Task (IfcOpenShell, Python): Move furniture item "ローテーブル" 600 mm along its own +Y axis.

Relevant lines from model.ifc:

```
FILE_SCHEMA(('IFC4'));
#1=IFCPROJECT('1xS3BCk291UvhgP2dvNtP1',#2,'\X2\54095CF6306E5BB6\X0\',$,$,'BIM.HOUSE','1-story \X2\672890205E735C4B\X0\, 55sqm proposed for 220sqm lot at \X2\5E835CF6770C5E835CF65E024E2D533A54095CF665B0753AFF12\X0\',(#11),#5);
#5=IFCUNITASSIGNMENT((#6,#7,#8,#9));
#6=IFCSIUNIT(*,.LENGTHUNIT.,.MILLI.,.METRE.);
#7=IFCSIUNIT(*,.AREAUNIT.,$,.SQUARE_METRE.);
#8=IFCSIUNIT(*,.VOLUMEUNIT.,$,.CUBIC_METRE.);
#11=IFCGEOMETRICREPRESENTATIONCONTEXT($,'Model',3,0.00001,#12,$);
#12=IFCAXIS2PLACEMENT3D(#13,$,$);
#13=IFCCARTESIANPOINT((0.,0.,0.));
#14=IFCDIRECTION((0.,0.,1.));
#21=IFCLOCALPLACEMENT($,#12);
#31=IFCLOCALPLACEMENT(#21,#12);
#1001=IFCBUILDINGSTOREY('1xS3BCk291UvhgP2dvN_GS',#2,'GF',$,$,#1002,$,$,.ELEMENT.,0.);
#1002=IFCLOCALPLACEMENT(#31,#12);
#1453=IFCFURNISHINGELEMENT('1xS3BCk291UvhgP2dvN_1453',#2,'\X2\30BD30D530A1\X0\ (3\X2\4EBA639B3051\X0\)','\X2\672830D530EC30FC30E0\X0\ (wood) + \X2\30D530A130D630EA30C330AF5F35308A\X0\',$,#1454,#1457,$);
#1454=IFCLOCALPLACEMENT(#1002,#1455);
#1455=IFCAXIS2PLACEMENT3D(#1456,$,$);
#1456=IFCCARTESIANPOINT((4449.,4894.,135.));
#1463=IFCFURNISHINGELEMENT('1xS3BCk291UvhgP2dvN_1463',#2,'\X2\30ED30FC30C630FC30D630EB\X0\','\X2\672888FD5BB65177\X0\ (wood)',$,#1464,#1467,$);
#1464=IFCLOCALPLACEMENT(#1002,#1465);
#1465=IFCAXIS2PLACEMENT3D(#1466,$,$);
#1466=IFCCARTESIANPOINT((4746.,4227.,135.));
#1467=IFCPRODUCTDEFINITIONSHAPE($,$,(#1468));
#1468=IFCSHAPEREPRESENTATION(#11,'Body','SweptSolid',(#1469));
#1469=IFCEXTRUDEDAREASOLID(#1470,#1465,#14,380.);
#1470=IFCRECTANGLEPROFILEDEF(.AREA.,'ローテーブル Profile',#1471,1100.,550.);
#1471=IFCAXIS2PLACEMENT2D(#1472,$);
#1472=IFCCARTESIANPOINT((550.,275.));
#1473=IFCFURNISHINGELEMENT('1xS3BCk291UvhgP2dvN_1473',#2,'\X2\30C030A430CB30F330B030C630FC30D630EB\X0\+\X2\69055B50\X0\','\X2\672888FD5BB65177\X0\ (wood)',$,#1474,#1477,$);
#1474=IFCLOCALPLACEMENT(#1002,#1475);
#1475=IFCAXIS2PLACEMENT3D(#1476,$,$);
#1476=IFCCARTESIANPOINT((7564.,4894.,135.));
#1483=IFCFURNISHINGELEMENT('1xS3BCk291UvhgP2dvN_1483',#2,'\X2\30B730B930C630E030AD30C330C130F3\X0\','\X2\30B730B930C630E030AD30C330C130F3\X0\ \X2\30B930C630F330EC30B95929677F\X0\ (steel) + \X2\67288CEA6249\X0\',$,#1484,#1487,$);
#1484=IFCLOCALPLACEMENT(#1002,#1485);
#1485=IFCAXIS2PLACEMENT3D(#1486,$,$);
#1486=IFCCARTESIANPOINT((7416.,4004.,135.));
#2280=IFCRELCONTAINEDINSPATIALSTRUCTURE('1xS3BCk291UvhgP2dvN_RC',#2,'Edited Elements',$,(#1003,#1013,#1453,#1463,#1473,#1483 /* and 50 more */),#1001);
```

```python
import ifcopenshell
import ifcopenshell.api.geometry
import ifcopenshell.util.placement

model = ifcopenshell.open("model.ifc")

item = model.by_guid("1xS3BCk291UvhgP2dvN_1463")
matrix = ifcopenshell.util.placement.get_local_placement(item.ObjectPlacement)
matrix[:3, 3] += matrix[:3, 1] * 600.0
ifcopenshell.api.geometry.edit_object_placement(model, product=item, matrix=matrix, is_si=False)

print(ifcopenshell.util.placement.get_local_placement(item.ObjectPlacement).round(3) + 0.0)

model.write("model-out.ifc")
```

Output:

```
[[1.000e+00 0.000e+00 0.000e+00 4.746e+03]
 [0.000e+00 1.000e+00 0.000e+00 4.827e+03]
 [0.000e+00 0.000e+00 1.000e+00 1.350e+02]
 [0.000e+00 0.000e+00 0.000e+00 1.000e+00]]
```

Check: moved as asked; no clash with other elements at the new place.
